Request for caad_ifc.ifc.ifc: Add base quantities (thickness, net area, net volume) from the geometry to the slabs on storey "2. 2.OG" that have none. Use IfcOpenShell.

First a look at what the model holds.

```python
import ifcopenshell
import ifcopenshell.util.element
import ifcopenshell.util.unit

model = ifcopenshell.open("caad_ifc.ifc.ifc")
print(model.schema)
for unit_type in ("LENGTHUNIT", "AREAUNIT", "VOLUMEUNIT"):
    print(unit_type, ifcopenshell.util.unit.calculate_unit_scale(model, unit_type))
storey = next(s for s in model.by_type("IfcBuildingStorey") if s.Name == "2. 2.OG")
slabs = [e for e in ifcopenshell.util.element.get_decomposition(storey) if e.is_a("IfcSlab")]
for e in sorted(slabs, key=lambda e: e.id()):
    print(e.id(), e.is_a(), e.Name, list(ifcopenshell.util.element.get_psets(e, qtos_only=True)), sep=" | ")
```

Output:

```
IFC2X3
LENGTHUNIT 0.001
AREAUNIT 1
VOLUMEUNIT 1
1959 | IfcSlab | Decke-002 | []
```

```python
import ifcopenshell
import ifcopenshell.api.pset
import ifcopenshell.geom
import ifcopenshell.util.element
import ifcopenshell.util.shape
import ifcopenshell.util.unit

model = ifcopenshell.open("caad_ifc.ifc.ifc")
unit_scale = ifcopenshell.util.unit.calculate_unit_scale(model)
area_scale = ifcopenshell.util.unit.calculate_unit_scale(model, "AREAUNIT")
volume_scale = ifcopenshell.util.unit.calculate_unit_scale(model, "VOLUMEUNIT")
settings = ifcopenshell.geom.settings()

storey = next(s for s in model.by_type("IfcBuildingStorey") if s.Name == "2. 2.OG")
slabs = [e for e in ifcopenshell.util.element.get_decomposition(storey) if e.is_a("IfcSlab")]

for e in sorted(slabs, key=lambda e: e.id()):
    if ifcopenshell.util.element.get_psets(e, qtos_only=True, should_inherit=False):
        continue
    # Geometry comes back in metres, in the element's own axes.
    shape = ifcopenshell.geom.create_shape(settings, e)
    values = {
        "Width": ifcopenshell.util.shape.get_z(shape.geometry) / unit_scale,
        "NetArea": ifcopenshell.util.shape.get_footprint_area(shape.geometry) / area_scale,
        "NetVolume": ifcopenshell.util.shape.get_volume(shape.geometry) / volume_scale,
    }
    qto = ifcopenshell.api.pset.add_qto(model, product=e, name="BaseQuantities")
    ifcopenshell.api.pset.edit_qto(model, qto=qto, properties=values)
    print(e.id(), {k: round(v, 3) for k, v in values.items()})

model.write("caad_ifc.ifc_rev.ifc")
```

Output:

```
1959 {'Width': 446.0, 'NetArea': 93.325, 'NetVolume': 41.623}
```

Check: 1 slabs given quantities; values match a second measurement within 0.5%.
